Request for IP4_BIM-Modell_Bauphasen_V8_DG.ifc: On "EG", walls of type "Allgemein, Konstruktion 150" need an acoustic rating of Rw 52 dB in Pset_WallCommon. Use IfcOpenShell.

First a look at what the model holds.

```python
import ifcopenshell
import ifcopenshell.util.element

model = ifcopenshell.open("IP4_BIM-Modell_Bauphasen_V8_DG.ifc")
print(model.schema)
storey = next(s for s in model.by_type("IfcBuildingStorey") if s.Name == "EG")
walls = [e for e in ifcopenshell.util.element.get_decomposition(storey) if e.is_a("IfcWall")]
seen = {}
for e in walls:
    element_type = ifcopenshell.util.element.get_type(e)
    key = (element_type.Name if element_type != e and element_type else None, ifcopenshell.util.element.get_pset(e, "Pset_WallCommon", "AcousticRating"))
    seen[key] = seen.get(key, 0) + 1
for (name, value), count in sorted(seen.items(), key=str):
    print(count, "x", name, "|", value)
```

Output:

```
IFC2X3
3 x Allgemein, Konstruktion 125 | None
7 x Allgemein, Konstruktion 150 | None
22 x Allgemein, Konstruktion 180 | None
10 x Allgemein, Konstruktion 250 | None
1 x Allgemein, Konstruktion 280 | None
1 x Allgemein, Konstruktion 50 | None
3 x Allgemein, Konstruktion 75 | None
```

```python
import ifcopenshell
import ifcopenshell.api.pset
import ifcopenshell.util.element

model = ifcopenshell.open("IP4_BIM-Modell_Bauphasen_V8_DG.ifc")

storey = next(s for s in model.by_type("IfcBuildingStorey") if s.Name == "EG")
walls = [e for e in ifcopenshell.util.element.get_decomposition(storey) if e.is_a("IfcWall")]

count = 0
for e in walls:
    element_type = ifcopenshell.util.element.get_type(e)
    if element_type in (None, e) or element_type.Name != "Allgemein, Konstruktion 150":
        continue
    # add_pset returns the element's existing set when there is one.
    pset = ifcopenshell.api.pset.add_pset(model, product=e, name="Pset_WallCommon")
    ifcopenshell.api.pset.edit_pset(model, pset=pset, properties={"AcousticRating": "Rw 52 dB"})
    count += 1

print(count, "walls updated")

model.write("IP4_BIM-Modell_Bauphasen_V8_DG_edited.ifc")
```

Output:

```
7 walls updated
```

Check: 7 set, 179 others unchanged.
